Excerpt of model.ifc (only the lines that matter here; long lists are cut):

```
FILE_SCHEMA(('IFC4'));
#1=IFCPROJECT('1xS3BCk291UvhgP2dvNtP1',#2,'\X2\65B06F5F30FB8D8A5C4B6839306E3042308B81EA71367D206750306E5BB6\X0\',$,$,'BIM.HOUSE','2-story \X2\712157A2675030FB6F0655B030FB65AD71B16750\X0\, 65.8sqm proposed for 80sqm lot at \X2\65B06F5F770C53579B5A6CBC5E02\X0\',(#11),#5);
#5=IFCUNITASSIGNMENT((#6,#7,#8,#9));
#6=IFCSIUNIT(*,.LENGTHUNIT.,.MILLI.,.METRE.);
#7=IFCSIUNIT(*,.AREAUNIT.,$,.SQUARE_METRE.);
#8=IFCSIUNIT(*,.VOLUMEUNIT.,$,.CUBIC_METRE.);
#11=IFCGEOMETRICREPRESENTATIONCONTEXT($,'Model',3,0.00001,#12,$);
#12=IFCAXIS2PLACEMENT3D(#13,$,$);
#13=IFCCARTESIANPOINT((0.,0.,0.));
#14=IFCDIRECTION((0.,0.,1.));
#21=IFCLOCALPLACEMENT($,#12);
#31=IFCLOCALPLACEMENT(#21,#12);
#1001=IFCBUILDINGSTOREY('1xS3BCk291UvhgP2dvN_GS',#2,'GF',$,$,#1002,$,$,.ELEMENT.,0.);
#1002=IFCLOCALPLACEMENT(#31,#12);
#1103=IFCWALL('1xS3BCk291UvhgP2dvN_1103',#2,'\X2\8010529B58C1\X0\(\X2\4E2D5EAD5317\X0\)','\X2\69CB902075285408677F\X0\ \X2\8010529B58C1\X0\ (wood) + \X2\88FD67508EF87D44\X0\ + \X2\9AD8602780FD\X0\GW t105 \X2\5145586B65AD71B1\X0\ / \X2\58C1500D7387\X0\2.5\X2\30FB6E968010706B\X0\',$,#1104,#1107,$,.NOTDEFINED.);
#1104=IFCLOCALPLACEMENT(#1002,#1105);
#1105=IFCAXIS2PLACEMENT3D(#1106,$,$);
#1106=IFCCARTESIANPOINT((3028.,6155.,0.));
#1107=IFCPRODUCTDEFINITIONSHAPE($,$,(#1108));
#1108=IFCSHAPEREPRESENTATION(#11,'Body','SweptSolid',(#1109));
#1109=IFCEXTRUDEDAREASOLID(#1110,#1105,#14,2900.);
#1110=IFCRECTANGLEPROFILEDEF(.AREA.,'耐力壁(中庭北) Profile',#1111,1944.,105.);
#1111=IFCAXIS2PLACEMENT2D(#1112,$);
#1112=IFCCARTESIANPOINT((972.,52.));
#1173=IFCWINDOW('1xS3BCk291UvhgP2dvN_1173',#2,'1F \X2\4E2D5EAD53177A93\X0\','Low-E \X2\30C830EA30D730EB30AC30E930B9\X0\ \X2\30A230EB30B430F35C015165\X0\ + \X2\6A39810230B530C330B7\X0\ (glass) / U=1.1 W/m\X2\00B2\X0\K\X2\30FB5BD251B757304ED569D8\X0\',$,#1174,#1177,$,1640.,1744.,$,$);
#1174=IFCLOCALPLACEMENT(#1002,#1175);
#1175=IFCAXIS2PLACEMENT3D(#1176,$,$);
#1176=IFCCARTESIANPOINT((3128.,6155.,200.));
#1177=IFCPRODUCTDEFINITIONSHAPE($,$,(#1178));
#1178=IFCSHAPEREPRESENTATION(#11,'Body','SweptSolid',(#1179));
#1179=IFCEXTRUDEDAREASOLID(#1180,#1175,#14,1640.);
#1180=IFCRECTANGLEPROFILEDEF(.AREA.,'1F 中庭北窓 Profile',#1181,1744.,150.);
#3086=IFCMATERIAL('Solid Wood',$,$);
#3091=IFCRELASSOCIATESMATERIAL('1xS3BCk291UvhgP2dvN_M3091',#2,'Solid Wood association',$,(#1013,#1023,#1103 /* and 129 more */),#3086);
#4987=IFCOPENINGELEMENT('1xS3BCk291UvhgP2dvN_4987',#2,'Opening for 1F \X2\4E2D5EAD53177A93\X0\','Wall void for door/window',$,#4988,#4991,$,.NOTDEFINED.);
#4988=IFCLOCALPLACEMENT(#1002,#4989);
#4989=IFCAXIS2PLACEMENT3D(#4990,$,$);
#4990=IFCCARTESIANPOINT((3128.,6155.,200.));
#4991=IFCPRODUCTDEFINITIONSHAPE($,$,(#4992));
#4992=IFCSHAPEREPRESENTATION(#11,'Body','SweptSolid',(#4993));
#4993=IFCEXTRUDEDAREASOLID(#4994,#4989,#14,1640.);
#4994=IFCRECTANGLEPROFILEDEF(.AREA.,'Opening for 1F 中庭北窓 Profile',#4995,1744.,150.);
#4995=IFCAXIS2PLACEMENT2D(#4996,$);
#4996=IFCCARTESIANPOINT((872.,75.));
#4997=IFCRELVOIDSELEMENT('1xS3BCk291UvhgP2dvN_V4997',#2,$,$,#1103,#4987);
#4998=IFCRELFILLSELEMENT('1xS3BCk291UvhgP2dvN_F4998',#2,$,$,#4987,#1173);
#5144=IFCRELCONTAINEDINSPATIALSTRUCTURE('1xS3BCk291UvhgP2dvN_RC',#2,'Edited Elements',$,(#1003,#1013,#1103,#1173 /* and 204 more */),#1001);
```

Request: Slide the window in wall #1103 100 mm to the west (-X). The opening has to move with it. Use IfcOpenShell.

```python
import ifcopenshell
import ifcopenshell.api.geometry
import ifcopenshell.util.placement
import ifcopenshell.util.unit

model = ifcopenshell.open("model.ifc")
unit_scale = ifcopenshell.util.unit.calculate_unit_scale(model)

window = model.by_guid("1xS3BCk291UvhgP2dvN_1173")
opening = window.FillsVoids[0].RelatingOpeningElement
wall = opening.VoidsElements[0].RelatingBuildingElement

wall_matrix = ifcopenshell.util.placement.get_local_placement(wall.ObjectPlacement)
shift = wall_matrix[:3, 0] * -0.1 / unit_scale
before = ifcopenshell.util.placement.get_local_placement(window.ObjectPlacement)[:3, 3].copy()

# The window is not placed relative to its opening, so move both.
for product in (opening, window):
    matrix = ifcopenshell.util.placement.get_local_placement(product.ObjectPlacement)
    matrix[:3, 3] += shift
    ifcopenshell.api.geometry.edit_object_placement(model, product=product, matrix=matrix, is_si=False)

after = ifcopenshell.util.placement.get_local_placement(window.ObjectPlacement)[:3, 3]
print("window moved by", (after - before).round(3) + 0.0)

model.write("model_updated.ifc")
```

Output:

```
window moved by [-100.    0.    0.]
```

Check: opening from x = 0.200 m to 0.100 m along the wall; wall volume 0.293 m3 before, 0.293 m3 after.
